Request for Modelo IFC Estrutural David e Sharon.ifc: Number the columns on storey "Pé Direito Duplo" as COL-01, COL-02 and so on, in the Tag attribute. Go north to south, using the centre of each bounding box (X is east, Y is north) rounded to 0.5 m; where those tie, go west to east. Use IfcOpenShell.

First a look at what the model holds.

```python
import ifcopenshell
import ifcopenshell.util.element
import ifcopenshell.util.placement

model = ifcopenshell.open("Modelo IFC Estrutural David e Sharon.ifc")
print(model.schema)
storey = next(s for s in model.by_type("IfcBuildingStorey") if s.Name == "Pé Direito Duplo")
columns = [e for e in ifcopenshell.util.element.get_decomposition(storey) if e.is_a("IfcColumn")]
for e in sorted(columns, key=lambda e: e.id()):
    origin = ifcopenshell.util.placement.get_local_placement(e.ObjectPlacement)[:3, 3]
    print(e.id(), e.Tag, e.Name, origin.round(2) + 0.0, sep=" | ")
```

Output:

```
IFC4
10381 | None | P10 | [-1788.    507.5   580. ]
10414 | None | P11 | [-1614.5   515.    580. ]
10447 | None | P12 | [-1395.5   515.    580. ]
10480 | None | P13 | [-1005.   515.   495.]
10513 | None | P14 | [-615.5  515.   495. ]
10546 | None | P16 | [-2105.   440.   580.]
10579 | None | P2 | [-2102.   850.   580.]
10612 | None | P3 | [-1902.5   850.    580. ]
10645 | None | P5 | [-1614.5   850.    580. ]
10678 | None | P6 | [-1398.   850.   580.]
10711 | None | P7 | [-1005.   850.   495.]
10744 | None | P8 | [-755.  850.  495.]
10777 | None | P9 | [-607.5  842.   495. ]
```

```python
import ifcopenshell
import ifcopenshell.geom
import ifcopenshell.util.element
import ifcopenshell.util.shape

model = ifcopenshell.open("Modelo IFC Estrutural David e Sharon.ifc")
settings = ifcopenshell.geom.settings()
settings.set("use-world-coords", True)


def centre(element):
    shape = ifcopenshell.geom.create_shape(settings, element)
    return ifcopenshell.util.shape.get_bbox_centroid(shape.geometry)


storey = next(s for s in model.by_type("IfcBuildingStorey") if s.Name == "Pé Direito Duplo")
columns = [e for e in ifcopenshell.util.element.get_decomposition(storey) if e.is_a("IfcColumn")]

# Insertion points can sit at a corner or the storey origin, so sort by the geometry (in metres).
centres = {e: centre(e) for e in columns}
columns.sort(key=lambda e: (-round(centres[e][1] / 0.5), centres[e][0]))

for i, e in enumerate(columns, start=1):
    number = f"COL-{i:02d}"
    e.Tag = number
    print(e.id(), number)

model.write("Modelo IFC Estrutural David e Sharon_updated.ifc")
```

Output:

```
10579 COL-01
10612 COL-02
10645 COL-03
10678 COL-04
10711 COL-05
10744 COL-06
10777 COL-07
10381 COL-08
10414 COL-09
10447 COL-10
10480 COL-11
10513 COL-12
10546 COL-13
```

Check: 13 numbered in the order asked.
